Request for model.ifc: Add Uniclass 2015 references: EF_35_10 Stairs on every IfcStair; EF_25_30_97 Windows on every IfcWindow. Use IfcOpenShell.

First a look at what the model holds.

```python
import ifcopenshell

model = ifcopenshell.open("model.ifc")
print(model.schema)
print("classifications:", [c.Name for c in model.by_type("IfcClassification")])
for ifc_class in ("IfcDoor", "IfcRoof", "IfcStair", "IfcWall", "IfcWindow"):
    print(ifc_class, len(model.by_type(ifc_class)))
```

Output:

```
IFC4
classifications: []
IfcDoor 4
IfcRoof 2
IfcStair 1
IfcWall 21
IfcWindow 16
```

```python
import ifcopenshell
import ifcopenshell.api.classification

model = ifcopenshell.open("model.ifc")

system = ifcopenshell.api.classification.add_classification(model, classification="Uniclass 2015")

codes = {
    "IfcStair": ("EF_35_10", "Stairs"),
    "IfcWindow": ("EF_25_30_97", "Windows"),
}
for ifc_class, (code, name) in codes.items():
    products = model.by_type(ifc_class)
    ifcopenshell.api.classification.add_reference(
        model, products=products, classification=system, identification=code, name=name
    )
    print(code, len(products))

model.write("model_edited.ifc")
```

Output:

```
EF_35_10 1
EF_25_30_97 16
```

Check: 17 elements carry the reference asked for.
